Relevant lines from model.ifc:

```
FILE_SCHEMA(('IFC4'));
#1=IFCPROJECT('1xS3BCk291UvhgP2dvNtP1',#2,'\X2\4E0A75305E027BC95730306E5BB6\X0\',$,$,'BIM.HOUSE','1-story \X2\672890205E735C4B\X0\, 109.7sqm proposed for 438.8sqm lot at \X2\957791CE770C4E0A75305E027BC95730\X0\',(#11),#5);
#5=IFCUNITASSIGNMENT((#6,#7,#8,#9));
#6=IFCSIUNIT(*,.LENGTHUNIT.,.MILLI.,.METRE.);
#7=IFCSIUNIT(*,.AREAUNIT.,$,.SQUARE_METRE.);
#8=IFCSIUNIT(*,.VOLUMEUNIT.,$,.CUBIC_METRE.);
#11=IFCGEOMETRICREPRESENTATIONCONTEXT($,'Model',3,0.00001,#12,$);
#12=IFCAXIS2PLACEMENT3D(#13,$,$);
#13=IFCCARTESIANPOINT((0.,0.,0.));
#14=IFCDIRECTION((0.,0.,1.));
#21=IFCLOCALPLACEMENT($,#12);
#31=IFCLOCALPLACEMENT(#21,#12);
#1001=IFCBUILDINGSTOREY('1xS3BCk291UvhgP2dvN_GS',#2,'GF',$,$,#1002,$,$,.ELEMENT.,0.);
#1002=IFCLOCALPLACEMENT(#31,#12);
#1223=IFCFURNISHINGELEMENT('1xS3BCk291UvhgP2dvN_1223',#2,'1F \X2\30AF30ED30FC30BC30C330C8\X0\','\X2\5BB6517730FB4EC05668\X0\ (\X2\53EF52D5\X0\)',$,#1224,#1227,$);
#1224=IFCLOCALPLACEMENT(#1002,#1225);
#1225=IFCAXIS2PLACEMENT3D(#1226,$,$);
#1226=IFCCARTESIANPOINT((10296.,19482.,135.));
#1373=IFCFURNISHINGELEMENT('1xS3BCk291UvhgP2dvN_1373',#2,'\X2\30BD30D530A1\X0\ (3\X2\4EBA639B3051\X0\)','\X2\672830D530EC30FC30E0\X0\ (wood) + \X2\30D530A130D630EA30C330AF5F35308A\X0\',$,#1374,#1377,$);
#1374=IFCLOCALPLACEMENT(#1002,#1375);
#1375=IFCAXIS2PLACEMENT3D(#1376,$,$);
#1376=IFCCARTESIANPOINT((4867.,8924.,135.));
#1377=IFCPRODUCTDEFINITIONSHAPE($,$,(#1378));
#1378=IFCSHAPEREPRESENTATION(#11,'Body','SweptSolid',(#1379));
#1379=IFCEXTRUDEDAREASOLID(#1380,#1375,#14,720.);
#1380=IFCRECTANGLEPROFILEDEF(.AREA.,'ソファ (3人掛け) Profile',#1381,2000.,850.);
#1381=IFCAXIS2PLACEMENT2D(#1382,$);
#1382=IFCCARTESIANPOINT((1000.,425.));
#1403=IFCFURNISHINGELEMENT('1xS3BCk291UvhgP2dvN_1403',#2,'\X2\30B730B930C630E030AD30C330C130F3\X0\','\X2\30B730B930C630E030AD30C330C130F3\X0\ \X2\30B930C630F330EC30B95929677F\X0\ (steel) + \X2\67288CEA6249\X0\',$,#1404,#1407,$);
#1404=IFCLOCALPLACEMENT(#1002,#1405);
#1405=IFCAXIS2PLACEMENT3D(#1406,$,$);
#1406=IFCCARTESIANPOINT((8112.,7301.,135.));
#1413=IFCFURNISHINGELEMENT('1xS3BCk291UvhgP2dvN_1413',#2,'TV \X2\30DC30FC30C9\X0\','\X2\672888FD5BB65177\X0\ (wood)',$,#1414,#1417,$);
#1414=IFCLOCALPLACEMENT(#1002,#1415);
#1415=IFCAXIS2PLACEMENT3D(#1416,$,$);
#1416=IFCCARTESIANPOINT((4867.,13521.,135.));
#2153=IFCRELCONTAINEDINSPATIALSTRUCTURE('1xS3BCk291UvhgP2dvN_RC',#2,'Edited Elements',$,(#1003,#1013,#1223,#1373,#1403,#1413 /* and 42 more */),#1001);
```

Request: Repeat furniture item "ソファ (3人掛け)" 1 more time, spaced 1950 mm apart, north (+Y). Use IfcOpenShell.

```python
import numpy as np
import ifcopenshell
import ifcopenshell.api.geometry
import ifcopenshell.api.root
import ifcopenshell.util.element
import ifcopenshell.util.placement
import ifcopenshell.util.unit

model = ifcopenshell.open("model.ifc")
unit_scale = ifcopenshell.util.unit.calculate_unit_scale(model)


def reuse_history(source, copy):
    """copy_class also copies each property set's owner history, people and application; keep the originals."""
    for rel in copy.IsDefinedBy:
        if rel.is_a("IfcRelDefinesByProperties") and (history := rel.RelatingPropertyDefinition.OwnerHistory):
            rel.RelatingPropertyDefinition.OwnerHistory = source.OwnerHistory
            ifcopenshell.util.element.remove_deep2(model, history)


source = model.by_guid("1xS3BCk291UvhgP2dvN_1373")
base = ifcopenshell.util.placement.get_local_placement(source.ObjectPlacement)
step = np.array([0.0, 1.0, 0.0]) * 1.95 / unit_scale

for i in range(1, 2):
    copy = ifcopenshell.api.root.copy_class(model, product=source)
    copy.Representation = ifcopenshell.util.element.copy_deep(
        model, source.Representation, exclude=["IfcGeometricRepresentationContext", "IfcRepresentationMap"]
    )
    reuse_history(source, copy)
    matrix = base.copy()
    matrix[:3, 3] += i * step
    print("added at", matrix[:3, 3].round(3) + 0.0)
    ifcopenshell.api.geometry.edit_object_placement(model, product=copy, matrix=matrix, is_si=False)

model.write("model-out.ifc")
```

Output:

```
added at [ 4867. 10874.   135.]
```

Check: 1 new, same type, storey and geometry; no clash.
